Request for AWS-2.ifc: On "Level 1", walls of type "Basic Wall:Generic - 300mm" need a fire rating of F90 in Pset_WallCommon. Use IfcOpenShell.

First a look at what the model holds.

```python
import ifcopenshell
import ifcopenshell.util.element

model = ifcopenshell.open("AWS-2.ifc")
print(model.schema)
storey = next(s for s in model.by_type("IfcBuildingStorey") if s.Name == "Level 1")
walls = [e for e in ifcopenshell.util.element.get_decomposition(storey) if e.is_a("IfcWall")]
seen = {}
for e in walls:
    element_type = ifcopenshell.util.element.get_type(e)
    key = (element_type.Name if element_type != e and element_type else None, ifcopenshell.util.element.get_pset(e, "Pset_WallCommon", "FireRating"))
    seen[key] = seen.get(key, 0) + 1
for (name, value), count in sorted(seen.items(), key=str):
    print(count, "x", name, "|", value)
```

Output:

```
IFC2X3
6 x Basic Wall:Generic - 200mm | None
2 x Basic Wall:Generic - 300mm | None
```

```python
import ifcopenshell
import ifcopenshell.api.pset
import ifcopenshell.util.element

model = ifcopenshell.open("AWS-2.ifc")

storey = next(s for s in model.by_type("IfcBuildingStorey") if s.Name == "Level 1")
walls = [e for e in ifcopenshell.util.element.get_decomposition(storey) if e.is_a("IfcWall")]

count = 0
for e in walls:
    element_type = ifcopenshell.util.element.get_type(e)
    if element_type in (None, e) or element_type.Name != "Basic Wall:Generic - 300mm":
        continue
    # add_pset returns the element's existing set when there is one.
    pset = ifcopenshell.api.pset.add_pset(model, product=e, name="Pset_WallCommon")
    ifcopenshell.api.pset.edit_pset(model, pset=pset, properties={"FireRating": "F90"})
    count += 1

print(count, "walls updated")

model.write("AWS-2_edited.ifc")
```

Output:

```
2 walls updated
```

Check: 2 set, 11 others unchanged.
